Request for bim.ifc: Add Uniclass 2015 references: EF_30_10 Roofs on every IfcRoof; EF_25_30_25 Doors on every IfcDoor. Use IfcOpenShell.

First a look at what the model holds.

```python
import ifcopenshell

model = ifcopenshell.open("bim.ifc")
print(model.schema)
print("classifications:", [c.Name for c in model.by_type("IfcClassification")])
for ifc_class in ("IfcDoor", "IfcRoof", "IfcStair", "IfcWall", "IfcWindow"):
    print(ifc_class, len(model.by_type(ifc_class)))
```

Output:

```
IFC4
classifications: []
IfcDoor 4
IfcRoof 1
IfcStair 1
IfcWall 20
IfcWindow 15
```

```python
import ifcopenshell
import ifcopenshell.api.classification

model = ifcopenshell.open("bim.ifc")

system = ifcopenshell.api.classification.add_classification(model, classification="Uniclass 2015")

codes = {
    "IfcRoof": ("EF_30_10", "Roofs"),
    "IfcDoor": ("EF_25_30_25", "Doors"),
}
for ifc_class, (code, name) in codes.items():
    products = model.by_type(ifc_class)
    ifcopenshell.api.classification.add_reference(
        model, products=products, classification=system, identification=code, name=name
    )
    print(code, len(products))

model.write("bim_v2.ifc")
```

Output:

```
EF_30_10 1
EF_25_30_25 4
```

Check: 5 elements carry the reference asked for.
